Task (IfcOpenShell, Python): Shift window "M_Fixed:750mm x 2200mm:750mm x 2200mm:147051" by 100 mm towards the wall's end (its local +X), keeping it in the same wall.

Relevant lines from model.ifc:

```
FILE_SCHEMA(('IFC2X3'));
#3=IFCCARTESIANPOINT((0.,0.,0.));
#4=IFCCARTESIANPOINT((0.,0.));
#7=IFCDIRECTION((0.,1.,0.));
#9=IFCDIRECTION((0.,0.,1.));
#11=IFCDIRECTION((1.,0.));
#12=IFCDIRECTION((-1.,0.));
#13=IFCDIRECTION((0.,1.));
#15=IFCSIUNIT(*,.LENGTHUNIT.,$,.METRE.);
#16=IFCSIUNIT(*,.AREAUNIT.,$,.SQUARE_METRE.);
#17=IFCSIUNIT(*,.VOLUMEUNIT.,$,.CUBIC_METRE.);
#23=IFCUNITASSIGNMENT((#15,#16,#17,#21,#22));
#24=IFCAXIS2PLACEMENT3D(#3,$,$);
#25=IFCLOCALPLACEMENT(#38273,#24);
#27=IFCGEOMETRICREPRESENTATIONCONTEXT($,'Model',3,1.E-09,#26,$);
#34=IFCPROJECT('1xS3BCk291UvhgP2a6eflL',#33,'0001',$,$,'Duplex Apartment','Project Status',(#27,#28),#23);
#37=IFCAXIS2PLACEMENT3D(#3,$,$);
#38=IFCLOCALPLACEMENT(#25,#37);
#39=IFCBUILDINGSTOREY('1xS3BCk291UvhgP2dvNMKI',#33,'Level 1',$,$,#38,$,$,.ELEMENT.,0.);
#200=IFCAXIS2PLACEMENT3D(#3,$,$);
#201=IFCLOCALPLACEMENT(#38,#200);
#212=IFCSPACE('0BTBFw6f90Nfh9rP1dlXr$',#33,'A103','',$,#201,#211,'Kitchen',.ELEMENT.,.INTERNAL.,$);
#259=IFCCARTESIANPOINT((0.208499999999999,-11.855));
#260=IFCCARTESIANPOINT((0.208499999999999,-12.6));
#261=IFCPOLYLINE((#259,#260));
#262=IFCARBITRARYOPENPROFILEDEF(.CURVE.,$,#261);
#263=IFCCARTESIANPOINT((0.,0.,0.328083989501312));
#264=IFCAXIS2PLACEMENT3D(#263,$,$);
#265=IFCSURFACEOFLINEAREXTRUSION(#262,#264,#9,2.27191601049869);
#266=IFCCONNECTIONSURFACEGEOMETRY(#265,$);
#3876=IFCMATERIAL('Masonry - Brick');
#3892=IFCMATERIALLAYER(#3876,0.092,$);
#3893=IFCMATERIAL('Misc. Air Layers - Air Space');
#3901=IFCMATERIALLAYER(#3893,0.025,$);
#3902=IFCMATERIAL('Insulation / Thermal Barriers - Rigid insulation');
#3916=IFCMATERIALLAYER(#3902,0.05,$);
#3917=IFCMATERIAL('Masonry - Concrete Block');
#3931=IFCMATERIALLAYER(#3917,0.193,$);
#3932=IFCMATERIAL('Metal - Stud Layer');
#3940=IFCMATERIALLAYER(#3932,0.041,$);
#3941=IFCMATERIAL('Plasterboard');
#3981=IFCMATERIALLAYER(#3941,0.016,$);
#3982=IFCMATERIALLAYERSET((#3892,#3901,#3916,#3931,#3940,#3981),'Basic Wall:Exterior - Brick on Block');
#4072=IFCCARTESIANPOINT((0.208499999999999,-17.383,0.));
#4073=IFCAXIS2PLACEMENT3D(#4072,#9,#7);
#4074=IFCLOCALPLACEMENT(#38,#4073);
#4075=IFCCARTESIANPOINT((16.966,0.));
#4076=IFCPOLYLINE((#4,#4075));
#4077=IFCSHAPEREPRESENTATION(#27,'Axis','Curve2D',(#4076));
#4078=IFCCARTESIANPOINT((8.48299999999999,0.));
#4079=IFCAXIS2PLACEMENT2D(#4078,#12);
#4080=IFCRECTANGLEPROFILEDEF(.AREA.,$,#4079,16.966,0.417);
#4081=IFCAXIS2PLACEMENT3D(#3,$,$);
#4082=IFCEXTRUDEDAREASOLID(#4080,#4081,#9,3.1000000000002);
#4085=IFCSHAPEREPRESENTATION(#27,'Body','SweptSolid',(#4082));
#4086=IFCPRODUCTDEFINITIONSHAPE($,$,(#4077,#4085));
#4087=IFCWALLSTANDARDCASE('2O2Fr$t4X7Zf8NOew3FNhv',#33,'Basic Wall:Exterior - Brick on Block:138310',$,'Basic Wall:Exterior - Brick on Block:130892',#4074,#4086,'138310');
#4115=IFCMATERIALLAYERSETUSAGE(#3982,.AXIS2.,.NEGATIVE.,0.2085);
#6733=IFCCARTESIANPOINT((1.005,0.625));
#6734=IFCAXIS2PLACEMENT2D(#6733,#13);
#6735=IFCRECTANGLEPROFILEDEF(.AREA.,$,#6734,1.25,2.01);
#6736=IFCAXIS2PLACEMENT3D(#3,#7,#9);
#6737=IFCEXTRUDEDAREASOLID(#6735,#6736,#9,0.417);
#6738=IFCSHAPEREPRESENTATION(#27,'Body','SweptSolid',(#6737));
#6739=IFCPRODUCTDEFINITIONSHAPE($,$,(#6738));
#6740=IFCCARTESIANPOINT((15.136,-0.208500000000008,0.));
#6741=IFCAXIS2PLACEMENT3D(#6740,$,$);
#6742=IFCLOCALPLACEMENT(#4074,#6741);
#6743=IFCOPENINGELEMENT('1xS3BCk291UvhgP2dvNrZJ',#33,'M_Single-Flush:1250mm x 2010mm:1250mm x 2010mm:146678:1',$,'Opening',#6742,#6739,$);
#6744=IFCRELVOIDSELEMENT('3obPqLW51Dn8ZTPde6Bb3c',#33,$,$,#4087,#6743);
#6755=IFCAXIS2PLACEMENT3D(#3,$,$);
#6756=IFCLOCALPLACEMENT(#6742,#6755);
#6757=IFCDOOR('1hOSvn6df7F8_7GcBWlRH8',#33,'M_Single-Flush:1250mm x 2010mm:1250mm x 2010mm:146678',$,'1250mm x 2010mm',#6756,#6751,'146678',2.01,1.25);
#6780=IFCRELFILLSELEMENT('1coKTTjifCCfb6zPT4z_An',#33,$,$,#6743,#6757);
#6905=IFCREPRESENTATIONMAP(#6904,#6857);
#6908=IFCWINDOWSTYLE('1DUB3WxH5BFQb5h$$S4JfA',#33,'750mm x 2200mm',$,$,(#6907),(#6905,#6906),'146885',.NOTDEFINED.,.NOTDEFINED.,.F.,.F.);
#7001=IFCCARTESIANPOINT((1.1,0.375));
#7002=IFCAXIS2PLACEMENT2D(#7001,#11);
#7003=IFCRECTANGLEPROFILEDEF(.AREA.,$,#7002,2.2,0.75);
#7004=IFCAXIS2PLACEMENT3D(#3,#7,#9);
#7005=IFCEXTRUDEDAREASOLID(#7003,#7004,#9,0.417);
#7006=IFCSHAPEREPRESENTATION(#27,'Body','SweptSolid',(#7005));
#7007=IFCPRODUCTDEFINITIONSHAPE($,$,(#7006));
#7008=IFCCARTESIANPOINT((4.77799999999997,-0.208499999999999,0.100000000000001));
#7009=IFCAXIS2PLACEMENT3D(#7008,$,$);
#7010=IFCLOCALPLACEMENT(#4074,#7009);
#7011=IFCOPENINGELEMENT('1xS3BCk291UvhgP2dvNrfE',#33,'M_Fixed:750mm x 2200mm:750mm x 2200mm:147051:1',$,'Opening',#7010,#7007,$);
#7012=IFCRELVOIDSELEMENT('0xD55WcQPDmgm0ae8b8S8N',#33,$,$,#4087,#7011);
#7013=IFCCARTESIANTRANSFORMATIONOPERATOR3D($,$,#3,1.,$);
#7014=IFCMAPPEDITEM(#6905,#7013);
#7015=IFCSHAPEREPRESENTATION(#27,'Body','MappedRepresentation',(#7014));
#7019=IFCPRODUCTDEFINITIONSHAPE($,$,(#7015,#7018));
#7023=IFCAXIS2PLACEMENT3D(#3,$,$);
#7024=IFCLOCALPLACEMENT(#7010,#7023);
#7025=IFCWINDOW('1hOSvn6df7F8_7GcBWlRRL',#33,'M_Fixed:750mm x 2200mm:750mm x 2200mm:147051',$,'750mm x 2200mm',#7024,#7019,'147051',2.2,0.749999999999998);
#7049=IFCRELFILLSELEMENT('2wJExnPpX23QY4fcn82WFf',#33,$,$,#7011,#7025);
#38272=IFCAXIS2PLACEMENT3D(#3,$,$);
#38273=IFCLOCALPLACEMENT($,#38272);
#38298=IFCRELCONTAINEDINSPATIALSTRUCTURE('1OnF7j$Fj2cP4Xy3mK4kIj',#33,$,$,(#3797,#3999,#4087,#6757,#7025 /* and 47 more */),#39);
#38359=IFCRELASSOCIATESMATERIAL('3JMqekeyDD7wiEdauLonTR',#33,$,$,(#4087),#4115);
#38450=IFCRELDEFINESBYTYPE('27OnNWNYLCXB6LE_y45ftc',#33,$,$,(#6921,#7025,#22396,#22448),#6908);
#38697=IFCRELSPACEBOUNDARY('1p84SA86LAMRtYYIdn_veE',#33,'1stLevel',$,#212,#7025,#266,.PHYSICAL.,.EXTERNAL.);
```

```python
import numpy as np
import ifcopenshell
import ifcopenshell.api.geometry
import ifcopenshell.util.placement

model = ifcopenshell.open("model.ifc")

window = model.by_id(7025)
opening = window.FillsVoids[0].RelatingOpeningElement
wall = opening.VoidsElements[0].RelatingBuildingElement

wall_matrix = ifcopenshell.util.placement.get_local_placement(wall.ObjectPlacement)
shift = wall_matrix[:3, 0] * 0.1
before = ifcopenshell.util.placement.get_local_placement(window.ObjectPlacement)[:3, 3].copy()

# The window is placed relative to its opening, so it follows when the opening moves.
matrix = ifcopenshell.util.placement.get_local_placement(opening.ObjectPlacement)
matrix[:3, 3] += shift
ifcopenshell.api.geometry.edit_object_placement(
    model, product=opening, matrix=matrix, is_si=False, should_transform_children=True
)

# Space boundary surfaces are stored in each space's coordinates; move them too.
for rel in window.ProvidesBoundaries:
    if not rel.ConnectionGeometry:
        continue
    surface = rel.ConnectionGeometry.SurfaceOnRelatingElement
    space_matrix = ifcopenshell.util.placement.get_local_placement(rel.RelatingSpace.ObjectPlacement)
    point = np.array(surface.Position.Location.Coordinates) + space_matrix[:3, :3].T @ shift
    surface.Position = model.createIfcAxis2Placement3D(
        model.createIfcCartesianPoint(point.tolist()), surface.Position.Axis, surface.Position.RefDirection
    )

after = ifcopenshell.util.placement.get_local_placement(window.ObjectPlacement)[:3, 3]
print("window moved by", (after - before).round(3) + 0.0)

model.write("model_v2.ifc")
```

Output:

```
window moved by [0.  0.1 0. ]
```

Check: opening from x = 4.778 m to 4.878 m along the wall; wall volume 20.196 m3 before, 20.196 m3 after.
